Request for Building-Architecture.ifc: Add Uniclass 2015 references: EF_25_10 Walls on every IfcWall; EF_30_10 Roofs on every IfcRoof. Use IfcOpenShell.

First a look at what the model holds.

```python
import ifcopenshell

model = ifcopenshell.open("Building-Architecture.ifc")
print(model.schema)
print("classifications:", [c.Name for c in model.by_type("IfcClassification")])
for ifc_class in ("IfcDoor", "IfcRoof", "IfcStair", "IfcWall", "IfcWindow"):
    print(ifc_class, len(model.by_type(ifc_class)))
```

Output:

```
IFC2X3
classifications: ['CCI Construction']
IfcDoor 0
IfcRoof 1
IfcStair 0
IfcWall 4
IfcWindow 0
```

```python
import ifcopenshell
import ifcopenshell.api.classification

model = ifcopenshell.open("Building-Architecture.ifc")

# IFC2X3 requires Source and Edition and has no link from the project to the system.
system = model.create_entity("IfcClassification", Source="NBS", Edition="2015", Name="Uniclass 2015")

codes = {
    "IfcWall": ("EF_25_10", "Walls"),
    "IfcRoof": ("EF_30_10", "Roofs"),
}
for ifc_class, (code, name) in codes.items():
    products = model.by_type(ifc_class)
    ifcopenshell.api.classification.add_reference(
        model, products=products, classification=system, identification=code, name=name
    )
    print(code, len(products))

model.write("Building-Architecture_v2.ifc")
```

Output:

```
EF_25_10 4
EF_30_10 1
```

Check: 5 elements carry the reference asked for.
